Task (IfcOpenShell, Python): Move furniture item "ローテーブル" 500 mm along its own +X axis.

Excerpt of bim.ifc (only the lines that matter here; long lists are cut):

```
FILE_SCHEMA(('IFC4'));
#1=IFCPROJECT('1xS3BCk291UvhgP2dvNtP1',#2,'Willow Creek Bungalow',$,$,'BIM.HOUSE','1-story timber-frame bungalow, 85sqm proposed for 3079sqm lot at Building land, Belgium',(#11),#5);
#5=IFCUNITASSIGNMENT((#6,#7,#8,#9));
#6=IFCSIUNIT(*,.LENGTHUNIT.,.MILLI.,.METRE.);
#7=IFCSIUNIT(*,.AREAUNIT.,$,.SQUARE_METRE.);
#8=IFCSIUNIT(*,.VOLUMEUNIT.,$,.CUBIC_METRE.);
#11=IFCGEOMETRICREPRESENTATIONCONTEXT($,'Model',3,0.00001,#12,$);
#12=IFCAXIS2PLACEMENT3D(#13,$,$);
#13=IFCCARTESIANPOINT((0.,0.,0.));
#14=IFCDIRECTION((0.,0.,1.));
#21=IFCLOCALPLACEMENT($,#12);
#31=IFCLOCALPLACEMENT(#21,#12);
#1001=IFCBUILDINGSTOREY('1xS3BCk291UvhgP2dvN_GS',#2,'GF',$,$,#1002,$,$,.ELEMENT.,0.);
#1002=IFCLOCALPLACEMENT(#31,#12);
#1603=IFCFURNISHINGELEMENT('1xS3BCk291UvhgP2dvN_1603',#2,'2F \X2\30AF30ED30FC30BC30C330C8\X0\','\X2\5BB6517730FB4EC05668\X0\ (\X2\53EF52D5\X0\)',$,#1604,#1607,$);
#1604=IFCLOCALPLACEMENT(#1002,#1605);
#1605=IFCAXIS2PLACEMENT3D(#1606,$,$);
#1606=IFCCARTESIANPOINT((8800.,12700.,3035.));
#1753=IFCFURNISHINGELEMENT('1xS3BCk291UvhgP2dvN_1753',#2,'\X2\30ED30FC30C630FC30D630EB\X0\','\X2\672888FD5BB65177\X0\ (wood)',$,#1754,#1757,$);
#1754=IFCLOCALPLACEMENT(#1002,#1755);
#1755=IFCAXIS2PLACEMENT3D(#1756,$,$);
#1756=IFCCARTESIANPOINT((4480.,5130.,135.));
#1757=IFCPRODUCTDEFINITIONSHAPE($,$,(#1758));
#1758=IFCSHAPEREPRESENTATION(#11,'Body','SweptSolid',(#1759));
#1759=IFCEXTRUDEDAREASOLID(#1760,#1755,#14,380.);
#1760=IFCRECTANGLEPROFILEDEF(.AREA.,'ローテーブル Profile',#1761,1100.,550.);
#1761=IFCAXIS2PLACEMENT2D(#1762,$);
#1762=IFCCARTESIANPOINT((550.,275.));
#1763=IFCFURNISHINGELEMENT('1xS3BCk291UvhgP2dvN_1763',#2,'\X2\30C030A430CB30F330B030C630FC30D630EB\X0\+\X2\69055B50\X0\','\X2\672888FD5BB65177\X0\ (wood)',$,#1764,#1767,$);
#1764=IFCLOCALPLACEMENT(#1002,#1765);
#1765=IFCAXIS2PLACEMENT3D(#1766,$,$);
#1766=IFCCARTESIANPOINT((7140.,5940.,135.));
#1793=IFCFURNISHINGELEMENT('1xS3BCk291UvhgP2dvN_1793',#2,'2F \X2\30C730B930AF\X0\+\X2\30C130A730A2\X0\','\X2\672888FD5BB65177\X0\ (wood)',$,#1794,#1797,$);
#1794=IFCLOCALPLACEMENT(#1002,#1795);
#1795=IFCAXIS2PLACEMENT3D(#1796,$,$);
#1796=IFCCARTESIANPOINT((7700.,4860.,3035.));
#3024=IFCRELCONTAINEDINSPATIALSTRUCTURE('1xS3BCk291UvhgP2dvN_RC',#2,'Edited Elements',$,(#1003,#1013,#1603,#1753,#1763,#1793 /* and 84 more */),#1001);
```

```python
import ifcopenshell
import ifcopenshell.api.geometry
import ifcopenshell.util.placement
import ifcopenshell.util.unit

model = ifcopenshell.open("bim.ifc")
unit_scale = ifcopenshell.util.unit.calculate_unit_scale(model)

item = model.by_guid("1xS3BCk291UvhgP2dvN_1753")
matrix = ifcopenshell.util.placement.get_local_placement(item.ObjectPlacement)
matrix[:3, 3] += matrix[:3, 0] * 0.5 / unit_scale
ifcopenshell.api.geometry.edit_object_placement(model, product=item, matrix=matrix, is_si=False)

print(ifcopenshell.util.placement.get_local_placement(item.ObjectPlacement).round(3) + 0.0)

model.write("bim_updated.ifc")
```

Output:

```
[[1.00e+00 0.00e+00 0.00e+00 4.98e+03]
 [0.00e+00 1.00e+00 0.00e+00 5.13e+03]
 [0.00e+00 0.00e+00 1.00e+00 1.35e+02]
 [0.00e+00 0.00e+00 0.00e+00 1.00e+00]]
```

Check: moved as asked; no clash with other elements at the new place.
